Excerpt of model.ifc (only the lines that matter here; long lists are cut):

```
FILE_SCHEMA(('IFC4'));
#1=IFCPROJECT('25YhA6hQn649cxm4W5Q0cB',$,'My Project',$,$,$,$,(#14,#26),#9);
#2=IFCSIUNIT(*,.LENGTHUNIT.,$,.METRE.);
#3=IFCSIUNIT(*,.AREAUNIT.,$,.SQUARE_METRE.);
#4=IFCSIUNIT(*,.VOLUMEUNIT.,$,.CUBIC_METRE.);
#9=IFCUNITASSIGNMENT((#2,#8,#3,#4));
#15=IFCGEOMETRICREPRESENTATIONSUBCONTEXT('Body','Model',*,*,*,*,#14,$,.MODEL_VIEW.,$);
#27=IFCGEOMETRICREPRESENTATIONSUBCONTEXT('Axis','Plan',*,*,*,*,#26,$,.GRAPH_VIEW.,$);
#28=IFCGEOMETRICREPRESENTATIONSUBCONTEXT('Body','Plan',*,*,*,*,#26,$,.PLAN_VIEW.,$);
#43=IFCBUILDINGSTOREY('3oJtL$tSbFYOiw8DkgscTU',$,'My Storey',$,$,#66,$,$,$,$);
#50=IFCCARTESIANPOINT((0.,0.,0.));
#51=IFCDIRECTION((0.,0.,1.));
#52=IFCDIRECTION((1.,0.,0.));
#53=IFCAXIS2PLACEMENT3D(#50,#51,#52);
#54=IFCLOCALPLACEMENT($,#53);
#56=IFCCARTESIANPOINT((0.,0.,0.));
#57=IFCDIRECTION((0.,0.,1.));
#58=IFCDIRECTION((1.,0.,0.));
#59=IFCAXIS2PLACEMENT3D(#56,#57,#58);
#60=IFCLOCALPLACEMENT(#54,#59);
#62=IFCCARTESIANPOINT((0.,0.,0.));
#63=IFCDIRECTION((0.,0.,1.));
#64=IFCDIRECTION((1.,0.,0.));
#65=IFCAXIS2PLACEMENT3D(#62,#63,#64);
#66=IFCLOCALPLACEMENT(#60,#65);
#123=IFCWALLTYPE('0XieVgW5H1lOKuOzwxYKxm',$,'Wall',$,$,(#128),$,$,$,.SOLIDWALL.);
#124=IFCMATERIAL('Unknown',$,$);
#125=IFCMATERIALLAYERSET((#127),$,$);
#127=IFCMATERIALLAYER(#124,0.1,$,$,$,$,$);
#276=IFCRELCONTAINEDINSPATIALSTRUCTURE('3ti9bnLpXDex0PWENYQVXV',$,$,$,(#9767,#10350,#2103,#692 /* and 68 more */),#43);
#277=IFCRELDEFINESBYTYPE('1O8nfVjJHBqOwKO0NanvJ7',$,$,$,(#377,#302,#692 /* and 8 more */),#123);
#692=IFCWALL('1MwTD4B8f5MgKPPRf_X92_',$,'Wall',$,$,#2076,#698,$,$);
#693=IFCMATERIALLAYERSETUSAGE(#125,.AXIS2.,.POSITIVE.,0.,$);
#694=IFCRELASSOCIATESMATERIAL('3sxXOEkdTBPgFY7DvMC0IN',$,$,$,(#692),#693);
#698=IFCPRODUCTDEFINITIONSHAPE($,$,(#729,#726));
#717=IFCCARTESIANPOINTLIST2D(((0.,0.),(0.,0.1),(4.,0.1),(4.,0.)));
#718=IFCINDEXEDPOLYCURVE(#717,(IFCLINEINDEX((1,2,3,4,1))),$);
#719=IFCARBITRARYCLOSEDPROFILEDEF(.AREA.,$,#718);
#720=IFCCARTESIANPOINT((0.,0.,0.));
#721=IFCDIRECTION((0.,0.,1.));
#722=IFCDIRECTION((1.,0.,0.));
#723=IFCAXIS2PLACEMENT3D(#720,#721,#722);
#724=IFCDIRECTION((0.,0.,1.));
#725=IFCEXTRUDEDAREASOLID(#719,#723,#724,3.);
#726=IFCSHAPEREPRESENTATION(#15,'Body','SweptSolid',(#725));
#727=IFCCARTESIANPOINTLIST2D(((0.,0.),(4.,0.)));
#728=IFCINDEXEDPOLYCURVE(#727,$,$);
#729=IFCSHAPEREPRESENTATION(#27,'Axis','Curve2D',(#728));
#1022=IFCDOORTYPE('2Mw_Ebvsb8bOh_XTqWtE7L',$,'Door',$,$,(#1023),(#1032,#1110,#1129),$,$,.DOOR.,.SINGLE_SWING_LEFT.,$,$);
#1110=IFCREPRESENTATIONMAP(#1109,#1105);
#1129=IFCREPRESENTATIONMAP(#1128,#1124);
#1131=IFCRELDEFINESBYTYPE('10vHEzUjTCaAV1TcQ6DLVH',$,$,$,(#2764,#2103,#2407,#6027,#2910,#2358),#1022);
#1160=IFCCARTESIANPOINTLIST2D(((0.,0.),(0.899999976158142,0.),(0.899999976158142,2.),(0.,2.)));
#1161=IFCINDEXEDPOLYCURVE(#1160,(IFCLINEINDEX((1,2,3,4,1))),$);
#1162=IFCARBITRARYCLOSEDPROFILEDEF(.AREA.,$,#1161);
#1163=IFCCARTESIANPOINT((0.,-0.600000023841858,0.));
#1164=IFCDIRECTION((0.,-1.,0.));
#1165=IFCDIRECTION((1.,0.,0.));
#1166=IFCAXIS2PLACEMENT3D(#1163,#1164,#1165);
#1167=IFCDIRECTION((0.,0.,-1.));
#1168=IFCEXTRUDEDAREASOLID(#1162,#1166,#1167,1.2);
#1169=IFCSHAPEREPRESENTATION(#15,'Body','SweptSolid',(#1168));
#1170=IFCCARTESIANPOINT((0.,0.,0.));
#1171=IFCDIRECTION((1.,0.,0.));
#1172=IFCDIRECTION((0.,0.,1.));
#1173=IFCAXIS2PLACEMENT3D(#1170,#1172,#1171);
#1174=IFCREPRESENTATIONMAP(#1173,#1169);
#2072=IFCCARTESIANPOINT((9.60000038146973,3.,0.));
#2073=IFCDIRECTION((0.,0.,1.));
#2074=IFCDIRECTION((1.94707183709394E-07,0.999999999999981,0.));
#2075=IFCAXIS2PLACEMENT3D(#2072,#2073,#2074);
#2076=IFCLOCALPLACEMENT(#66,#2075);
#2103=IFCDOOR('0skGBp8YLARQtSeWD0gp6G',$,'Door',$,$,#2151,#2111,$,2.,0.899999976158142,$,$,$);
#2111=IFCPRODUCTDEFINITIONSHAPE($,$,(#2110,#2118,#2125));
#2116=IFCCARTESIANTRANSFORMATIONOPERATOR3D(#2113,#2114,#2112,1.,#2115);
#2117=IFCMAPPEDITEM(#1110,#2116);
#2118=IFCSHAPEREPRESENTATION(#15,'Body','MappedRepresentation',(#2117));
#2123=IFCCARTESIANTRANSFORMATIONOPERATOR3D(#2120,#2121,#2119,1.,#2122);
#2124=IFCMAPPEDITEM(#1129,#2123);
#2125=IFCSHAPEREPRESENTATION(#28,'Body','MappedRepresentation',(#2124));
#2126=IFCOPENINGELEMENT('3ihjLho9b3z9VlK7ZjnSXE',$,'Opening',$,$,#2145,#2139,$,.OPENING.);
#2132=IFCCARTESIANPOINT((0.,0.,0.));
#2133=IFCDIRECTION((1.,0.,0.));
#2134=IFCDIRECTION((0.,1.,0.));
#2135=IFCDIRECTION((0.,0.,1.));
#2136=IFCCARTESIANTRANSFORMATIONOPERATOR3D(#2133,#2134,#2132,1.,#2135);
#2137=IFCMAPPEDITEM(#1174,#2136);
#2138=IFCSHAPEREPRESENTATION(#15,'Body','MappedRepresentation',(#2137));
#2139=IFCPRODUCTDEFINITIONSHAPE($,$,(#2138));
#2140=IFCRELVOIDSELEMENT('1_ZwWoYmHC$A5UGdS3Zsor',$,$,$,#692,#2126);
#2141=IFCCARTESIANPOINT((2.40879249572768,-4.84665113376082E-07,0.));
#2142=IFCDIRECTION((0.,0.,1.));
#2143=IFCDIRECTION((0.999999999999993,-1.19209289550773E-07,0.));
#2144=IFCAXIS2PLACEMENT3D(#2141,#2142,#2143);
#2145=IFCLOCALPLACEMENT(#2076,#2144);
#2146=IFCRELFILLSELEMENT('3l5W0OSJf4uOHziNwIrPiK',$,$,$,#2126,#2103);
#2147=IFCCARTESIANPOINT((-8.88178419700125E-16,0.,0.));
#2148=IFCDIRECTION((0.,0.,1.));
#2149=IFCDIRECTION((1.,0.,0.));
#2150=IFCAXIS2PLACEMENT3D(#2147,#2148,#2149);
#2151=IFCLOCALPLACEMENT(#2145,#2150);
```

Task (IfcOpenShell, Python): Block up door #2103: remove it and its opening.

```python
import ifcopenshell
import ifcopenshell.api.feature
import ifcopenshell.api.root
import ifcopenshell.geom
import ifcopenshell.util.shape

model = ifcopenshell.open("model.ifc")
settings = ifcopenshell.geom.settings()


def volume(element):
    """Net volume in cubic metres, openings subtracted."""
    shape = ifcopenshell.geom.create_shape(settings, element)
    return ifcopenshell.util.shape.get_volume(shape.geometry)


door = model.by_guid("0skGBp8YLARQtSeWD0gp6G")
opening = door.FillsVoids[0].RelatingOpeningElement
wall = opening.VoidsElements[0].RelatingBuildingElement
before = volume(wall)

ifcopenshell.api.root.remove_product(model, product=door)
ifcopenshell.api.feature.remove_feature(model, feature=opening)

after = volume(wall)

print(f"wall volume {before:.3f} -> {after:.3f} m3")

model.write("model_edited.ifc")
```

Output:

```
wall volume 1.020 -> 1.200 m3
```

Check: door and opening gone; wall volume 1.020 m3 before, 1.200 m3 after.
